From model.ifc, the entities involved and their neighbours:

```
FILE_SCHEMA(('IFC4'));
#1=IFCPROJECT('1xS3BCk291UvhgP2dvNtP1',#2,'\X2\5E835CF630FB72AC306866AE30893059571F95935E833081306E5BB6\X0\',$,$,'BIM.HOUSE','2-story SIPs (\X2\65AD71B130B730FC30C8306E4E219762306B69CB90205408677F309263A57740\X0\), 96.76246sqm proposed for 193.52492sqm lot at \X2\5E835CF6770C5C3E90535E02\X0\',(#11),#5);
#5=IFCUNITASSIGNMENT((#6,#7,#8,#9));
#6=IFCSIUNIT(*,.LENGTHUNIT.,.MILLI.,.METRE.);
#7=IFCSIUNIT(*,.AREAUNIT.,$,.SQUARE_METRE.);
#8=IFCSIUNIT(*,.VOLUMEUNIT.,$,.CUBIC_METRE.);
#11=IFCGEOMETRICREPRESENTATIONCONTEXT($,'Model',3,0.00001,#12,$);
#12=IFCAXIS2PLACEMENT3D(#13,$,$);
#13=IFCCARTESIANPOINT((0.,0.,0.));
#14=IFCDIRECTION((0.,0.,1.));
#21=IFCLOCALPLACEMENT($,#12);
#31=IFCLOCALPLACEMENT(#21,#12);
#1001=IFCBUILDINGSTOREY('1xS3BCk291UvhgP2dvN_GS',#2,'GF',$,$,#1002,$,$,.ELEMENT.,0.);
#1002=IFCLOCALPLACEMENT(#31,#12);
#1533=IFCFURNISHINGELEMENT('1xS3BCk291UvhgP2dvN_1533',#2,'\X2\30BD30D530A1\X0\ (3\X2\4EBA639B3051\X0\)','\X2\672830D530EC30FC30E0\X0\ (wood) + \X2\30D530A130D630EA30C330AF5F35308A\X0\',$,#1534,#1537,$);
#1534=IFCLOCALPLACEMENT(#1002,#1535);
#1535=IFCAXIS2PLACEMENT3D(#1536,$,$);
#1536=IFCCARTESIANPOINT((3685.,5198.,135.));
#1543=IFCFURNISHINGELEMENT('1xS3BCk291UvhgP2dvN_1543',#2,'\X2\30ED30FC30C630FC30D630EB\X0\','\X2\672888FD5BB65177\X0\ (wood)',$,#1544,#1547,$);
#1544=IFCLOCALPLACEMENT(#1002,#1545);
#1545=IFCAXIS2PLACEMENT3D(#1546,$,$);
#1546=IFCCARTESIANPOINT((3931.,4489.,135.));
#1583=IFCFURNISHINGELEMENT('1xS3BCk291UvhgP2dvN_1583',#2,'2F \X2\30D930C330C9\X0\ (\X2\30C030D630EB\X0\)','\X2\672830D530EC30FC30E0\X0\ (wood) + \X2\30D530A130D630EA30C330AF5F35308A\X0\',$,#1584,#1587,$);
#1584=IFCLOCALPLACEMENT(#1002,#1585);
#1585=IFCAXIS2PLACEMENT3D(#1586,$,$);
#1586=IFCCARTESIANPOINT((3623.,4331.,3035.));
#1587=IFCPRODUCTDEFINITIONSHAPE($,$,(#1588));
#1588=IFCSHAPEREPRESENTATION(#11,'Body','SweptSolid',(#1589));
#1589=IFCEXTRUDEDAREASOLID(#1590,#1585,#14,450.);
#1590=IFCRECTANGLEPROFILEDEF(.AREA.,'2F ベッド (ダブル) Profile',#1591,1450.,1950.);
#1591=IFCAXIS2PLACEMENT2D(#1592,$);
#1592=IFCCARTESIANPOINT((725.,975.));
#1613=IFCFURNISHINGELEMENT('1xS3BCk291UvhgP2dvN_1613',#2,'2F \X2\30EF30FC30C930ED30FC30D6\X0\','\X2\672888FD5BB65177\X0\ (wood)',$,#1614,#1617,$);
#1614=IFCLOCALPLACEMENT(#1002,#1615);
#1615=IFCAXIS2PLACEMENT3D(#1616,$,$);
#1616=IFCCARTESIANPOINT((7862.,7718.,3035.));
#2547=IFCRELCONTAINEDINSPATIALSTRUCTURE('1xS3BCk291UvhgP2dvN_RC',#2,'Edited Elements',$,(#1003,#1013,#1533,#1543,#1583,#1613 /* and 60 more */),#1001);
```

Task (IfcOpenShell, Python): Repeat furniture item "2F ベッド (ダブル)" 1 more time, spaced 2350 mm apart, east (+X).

```python
import numpy as np
import ifcopenshell
import ifcopenshell.api.geometry
import ifcopenshell.api.root
import ifcopenshell.util.element
import ifcopenshell.util.placement
import ifcopenshell.util.unit

model = ifcopenshell.open("model.ifc")
unit_scale = ifcopenshell.util.unit.calculate_unit_scale(model)


def reuse_history(source, copy):
    """copy_class also copies each property set's owner history, people and application; keep the originals."""
    for rel in copy.IsDefinedBy:
        if rel.is_a("IfcRelDefinesByProperties") and (history := rel.RelatingPropertyDefinition.OwnerHistory):
            rel.RelatingPropertyDefinition.OwnerHistory = source.OwnerHistory
            ifcopenshell.util.element.remove_deep2(model, history)


source = model.by_guid("1xS3BCk291UvhgP2dvN_1583")
base = ifcopenshell.util.placement.get_local_placement(source.ObjectPlacement)
step = np.array([1.0, 0.0, 0.0]) * 2.35 / unit_scale

for i in range(1, 2):
    copy = ifcopenshell.api.root.copy_class(model, product=source)
    copy.Representation = ifcopenshell.util.element.copy_deep(
        model, source.Representation, exclude=["IfcGeometricRepresentationContext", "IfcRepresentationMap"]
    )
    reuse_history(source, copy)
    matrix = base.copy()
    matrix[:3, 3] += i * step
    print("added at", matrix[:3, 3].round(3) + 0.0)
    ifcopenshell.api.geometry.edit_object_placement(model, product=copy, matrix=matrix, is_si=False)

model.write("model_updated.ifc")
```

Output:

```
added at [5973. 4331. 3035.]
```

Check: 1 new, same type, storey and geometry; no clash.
